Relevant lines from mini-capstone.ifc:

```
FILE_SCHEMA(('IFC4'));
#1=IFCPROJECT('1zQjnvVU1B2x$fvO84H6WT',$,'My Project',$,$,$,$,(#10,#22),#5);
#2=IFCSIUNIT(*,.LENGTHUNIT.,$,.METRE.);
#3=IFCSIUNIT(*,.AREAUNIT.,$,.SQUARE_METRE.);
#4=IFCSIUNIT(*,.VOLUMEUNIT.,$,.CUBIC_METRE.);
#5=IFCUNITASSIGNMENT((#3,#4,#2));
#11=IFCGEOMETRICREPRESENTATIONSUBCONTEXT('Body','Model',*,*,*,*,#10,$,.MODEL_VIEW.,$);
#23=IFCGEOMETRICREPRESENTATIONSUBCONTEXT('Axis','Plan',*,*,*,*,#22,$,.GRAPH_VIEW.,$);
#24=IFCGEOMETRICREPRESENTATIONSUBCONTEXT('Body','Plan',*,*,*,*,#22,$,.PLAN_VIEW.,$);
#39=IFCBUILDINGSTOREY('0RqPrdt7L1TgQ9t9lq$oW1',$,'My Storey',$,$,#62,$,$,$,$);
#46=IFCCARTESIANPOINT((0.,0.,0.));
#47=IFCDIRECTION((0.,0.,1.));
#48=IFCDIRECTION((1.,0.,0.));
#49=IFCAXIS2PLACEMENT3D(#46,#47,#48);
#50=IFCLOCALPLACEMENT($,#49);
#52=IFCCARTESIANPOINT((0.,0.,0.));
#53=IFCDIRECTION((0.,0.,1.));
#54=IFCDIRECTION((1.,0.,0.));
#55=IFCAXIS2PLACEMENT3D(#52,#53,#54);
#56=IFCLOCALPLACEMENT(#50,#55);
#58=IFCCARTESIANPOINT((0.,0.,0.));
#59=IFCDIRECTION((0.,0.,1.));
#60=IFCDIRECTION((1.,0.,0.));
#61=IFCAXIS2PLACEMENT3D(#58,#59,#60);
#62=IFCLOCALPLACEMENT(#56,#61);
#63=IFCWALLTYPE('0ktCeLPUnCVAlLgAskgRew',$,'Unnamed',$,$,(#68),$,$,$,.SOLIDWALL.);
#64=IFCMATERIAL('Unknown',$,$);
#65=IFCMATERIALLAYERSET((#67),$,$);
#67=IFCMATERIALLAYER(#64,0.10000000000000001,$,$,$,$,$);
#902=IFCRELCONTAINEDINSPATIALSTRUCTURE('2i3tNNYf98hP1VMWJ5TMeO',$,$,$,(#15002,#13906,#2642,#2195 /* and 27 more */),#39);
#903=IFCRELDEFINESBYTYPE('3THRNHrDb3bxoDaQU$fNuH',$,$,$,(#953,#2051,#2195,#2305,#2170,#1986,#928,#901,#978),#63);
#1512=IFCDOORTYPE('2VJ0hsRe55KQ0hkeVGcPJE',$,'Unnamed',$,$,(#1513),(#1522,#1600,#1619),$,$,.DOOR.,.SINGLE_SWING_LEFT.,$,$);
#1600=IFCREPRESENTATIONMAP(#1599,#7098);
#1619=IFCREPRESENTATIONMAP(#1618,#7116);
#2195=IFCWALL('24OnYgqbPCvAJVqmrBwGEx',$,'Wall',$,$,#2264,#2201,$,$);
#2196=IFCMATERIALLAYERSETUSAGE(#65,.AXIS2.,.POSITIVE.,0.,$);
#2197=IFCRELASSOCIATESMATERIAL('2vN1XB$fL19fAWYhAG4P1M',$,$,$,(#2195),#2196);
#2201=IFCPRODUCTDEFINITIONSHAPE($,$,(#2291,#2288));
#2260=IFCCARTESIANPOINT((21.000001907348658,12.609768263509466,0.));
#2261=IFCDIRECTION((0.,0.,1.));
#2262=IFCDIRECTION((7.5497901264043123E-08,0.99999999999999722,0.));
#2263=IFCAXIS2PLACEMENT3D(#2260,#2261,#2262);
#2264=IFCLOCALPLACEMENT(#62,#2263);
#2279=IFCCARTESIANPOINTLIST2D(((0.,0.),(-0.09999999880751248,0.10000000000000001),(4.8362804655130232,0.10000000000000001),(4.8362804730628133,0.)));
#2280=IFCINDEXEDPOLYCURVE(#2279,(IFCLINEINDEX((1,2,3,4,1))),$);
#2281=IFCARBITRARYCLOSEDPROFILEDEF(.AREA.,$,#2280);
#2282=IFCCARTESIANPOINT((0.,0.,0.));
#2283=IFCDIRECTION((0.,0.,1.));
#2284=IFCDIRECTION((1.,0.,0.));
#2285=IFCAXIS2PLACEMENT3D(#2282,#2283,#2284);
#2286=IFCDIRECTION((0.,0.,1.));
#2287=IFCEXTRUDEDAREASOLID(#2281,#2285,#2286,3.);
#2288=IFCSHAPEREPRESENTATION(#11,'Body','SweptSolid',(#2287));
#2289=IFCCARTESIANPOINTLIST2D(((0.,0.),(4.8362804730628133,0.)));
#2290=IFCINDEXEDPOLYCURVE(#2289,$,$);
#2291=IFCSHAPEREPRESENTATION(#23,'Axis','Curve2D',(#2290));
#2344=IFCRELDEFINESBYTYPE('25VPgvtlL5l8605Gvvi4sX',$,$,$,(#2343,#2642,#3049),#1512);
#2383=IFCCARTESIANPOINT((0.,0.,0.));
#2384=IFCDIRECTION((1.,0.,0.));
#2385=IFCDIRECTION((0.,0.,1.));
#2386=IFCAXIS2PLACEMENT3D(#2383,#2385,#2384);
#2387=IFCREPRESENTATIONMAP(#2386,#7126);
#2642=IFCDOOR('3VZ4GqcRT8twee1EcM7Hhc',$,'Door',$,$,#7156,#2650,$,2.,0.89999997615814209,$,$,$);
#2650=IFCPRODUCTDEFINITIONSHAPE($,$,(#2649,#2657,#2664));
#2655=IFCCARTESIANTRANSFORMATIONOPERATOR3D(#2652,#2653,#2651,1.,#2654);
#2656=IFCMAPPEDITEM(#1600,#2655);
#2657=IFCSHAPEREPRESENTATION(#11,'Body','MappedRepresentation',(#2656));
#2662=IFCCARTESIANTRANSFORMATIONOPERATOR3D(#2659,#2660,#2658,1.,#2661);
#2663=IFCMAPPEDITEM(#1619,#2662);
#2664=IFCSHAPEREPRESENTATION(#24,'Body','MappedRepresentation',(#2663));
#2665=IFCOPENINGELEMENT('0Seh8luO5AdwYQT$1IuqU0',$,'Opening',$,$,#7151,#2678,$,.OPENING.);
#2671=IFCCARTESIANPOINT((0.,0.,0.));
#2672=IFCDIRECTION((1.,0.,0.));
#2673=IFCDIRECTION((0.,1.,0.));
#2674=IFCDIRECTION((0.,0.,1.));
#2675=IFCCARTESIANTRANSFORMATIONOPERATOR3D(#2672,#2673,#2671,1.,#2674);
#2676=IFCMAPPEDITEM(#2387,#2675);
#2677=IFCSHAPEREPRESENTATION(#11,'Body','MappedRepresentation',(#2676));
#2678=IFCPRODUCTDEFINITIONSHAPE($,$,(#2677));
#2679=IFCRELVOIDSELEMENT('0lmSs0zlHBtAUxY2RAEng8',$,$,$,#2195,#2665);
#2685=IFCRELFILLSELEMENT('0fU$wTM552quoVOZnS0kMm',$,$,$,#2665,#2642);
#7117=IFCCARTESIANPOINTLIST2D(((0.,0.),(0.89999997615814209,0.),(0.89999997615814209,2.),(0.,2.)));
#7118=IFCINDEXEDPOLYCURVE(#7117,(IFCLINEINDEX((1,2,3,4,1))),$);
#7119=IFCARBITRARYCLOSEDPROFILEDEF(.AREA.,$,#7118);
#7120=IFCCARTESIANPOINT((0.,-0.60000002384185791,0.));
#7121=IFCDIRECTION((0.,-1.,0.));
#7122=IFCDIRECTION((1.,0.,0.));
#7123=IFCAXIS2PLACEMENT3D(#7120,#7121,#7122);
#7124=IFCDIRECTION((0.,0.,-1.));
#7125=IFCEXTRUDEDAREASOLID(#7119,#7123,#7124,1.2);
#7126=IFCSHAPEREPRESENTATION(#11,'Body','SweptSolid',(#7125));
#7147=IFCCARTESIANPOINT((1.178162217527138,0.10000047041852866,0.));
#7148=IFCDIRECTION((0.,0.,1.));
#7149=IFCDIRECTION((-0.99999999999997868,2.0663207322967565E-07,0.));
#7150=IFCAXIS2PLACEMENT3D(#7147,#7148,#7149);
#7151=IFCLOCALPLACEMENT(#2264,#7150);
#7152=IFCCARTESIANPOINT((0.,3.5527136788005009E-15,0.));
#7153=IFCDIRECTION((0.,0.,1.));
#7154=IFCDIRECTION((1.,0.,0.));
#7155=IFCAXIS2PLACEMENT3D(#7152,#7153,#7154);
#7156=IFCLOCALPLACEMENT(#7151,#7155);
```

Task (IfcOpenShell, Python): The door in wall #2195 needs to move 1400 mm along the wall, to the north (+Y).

```python
import ifcopenshell
import ifcopenshell.api.geometry
import ifcopenshell.util.placement
import ifcopenshell.util.unit

model = ifcopenshell.open("mini-capstone.ifc")
unit_scale = ifcopenshell.util.unit.calculate_unit_scale(model)

door = model.by_guid("3VZ4GqcRT8twee1EcM7Hhc")
opening = door.FillsVoids[0].RelatingOpeningElement
wall = opening.VoidsElements[0].RelatingBuildingElement

wall_matrix = ifcopenshell.util.placement.get_local_placement(wall.ObjectPlacement)
shift = wall_matrix[:3, 0] * 1.4 / unit_scale
before = ifcopenshell.util.placement.get_local_placement(door.ObjectPlacement)[:3, 3].copy()

# The door is placed relative to its opening, so it follows when the opening moves.
matrix = ifcopenshell.util.placement.get_local_placement(opening.ObjectPlacement)
matrix[:3, 3] += shift
ifcopenshell.api.geometry.edit_object_placement(
    model, product=opening, matrix=matrix, is_si=False, should_transform_children=True
)

after = ifcopenshell.util.placement.get_local_placement(door.ObjectPlacement)[:3, 3]
print("door moved by", (after - before).round(3) + 0.0)

model.write("mini-capstone_updated.ifc")
```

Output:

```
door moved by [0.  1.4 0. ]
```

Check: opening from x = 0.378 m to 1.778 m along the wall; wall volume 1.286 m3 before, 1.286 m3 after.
